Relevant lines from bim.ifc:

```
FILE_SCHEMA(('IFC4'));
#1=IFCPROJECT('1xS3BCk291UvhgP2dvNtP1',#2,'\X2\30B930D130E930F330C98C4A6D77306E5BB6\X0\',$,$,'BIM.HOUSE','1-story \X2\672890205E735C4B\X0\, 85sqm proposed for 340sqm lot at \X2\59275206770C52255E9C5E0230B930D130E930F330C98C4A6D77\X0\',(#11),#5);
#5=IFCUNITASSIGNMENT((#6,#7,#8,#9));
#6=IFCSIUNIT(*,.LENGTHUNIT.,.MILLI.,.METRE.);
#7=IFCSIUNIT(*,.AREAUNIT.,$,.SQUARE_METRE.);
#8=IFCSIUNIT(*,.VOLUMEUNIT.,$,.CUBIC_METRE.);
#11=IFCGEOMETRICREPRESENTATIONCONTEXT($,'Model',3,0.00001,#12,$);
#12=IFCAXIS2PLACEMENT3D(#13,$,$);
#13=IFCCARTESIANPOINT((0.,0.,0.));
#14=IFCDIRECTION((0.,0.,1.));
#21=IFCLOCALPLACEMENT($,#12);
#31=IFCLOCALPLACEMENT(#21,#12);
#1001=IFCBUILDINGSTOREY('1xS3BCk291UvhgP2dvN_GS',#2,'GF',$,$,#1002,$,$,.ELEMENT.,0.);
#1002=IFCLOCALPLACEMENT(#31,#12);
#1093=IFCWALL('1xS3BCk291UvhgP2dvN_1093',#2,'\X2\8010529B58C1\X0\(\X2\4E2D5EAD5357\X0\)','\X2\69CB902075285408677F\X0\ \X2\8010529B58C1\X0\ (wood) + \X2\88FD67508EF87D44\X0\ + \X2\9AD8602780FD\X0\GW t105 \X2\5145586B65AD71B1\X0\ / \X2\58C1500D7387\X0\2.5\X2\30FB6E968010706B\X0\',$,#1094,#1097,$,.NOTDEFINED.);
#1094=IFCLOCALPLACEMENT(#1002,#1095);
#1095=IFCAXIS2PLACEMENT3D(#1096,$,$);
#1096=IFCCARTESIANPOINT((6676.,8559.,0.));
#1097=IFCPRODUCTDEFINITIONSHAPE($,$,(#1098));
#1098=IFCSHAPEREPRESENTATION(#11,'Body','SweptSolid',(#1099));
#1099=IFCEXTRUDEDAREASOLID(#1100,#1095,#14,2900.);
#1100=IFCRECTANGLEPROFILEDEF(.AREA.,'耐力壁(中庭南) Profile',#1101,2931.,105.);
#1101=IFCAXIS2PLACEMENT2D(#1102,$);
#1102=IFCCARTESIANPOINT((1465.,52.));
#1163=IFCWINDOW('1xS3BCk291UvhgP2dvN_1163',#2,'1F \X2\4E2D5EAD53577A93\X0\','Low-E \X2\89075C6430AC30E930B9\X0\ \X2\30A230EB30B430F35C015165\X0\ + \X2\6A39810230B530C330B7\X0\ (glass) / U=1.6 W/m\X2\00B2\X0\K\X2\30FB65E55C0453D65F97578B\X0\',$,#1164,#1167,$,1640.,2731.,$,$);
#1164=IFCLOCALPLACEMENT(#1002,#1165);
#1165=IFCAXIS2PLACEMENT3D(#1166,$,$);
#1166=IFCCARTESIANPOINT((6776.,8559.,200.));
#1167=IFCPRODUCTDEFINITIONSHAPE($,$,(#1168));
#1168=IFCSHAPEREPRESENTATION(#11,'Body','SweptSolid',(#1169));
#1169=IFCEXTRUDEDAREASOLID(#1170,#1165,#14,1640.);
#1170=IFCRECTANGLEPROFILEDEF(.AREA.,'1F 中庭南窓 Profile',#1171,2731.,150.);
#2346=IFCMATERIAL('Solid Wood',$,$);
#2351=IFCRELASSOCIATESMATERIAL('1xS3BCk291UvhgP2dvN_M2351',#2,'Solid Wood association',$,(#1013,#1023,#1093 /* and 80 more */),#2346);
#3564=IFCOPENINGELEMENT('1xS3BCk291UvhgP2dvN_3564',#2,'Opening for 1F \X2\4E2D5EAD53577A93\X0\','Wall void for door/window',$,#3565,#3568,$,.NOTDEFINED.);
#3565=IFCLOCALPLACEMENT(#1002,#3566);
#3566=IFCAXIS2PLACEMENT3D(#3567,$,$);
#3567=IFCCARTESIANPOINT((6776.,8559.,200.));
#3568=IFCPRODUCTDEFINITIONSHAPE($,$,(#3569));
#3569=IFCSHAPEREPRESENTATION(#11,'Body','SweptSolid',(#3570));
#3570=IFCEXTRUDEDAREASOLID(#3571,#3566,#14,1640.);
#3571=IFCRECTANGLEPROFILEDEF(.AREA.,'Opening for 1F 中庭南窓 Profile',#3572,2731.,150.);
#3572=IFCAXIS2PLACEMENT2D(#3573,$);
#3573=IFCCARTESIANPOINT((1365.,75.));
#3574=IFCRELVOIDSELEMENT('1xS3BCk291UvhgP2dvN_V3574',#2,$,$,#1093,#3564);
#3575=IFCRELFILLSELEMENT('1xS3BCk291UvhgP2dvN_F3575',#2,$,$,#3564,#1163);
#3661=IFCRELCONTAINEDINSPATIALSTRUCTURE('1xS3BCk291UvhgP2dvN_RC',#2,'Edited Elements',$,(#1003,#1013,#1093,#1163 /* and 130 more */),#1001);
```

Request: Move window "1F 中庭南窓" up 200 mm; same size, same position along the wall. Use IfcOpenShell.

```python
import numpy as np
import ifcopenshell
import ifcopenshell.api.geometry
import ifcopenshell.util.placement
import ifcopenshell.util.unit

model = ifcopenshell.open("bim.ifc")
unit_scale = ifcopenshell.util.unit.calculate_unit_scale(model)

window = model.by_guid("1xS3BCk291UvhgP2dvN_1163")
opening = window.FillsVoids[0].RelatingOpeningElement
dz = 0.2 / unit_scale

shift = np.array([0.0, 0.0, dz])
# The window is not placed relative to its opening, so move both.
for product in (opening, window):
    matrix = ifcopenshell.util.placement.get_local_placement(product.ObjectPlacement)
    matrix[:3, 3] += shift
    ifcopenshell.api.geometry.edit_object_placement(model, product=product, matrix=matrix, is_si=False)

print(f"moved by {dz * unit_scale:+.3f} m")

model.write("bim_edited.ifc")
```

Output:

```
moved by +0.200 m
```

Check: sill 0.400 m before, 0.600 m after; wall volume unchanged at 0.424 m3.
